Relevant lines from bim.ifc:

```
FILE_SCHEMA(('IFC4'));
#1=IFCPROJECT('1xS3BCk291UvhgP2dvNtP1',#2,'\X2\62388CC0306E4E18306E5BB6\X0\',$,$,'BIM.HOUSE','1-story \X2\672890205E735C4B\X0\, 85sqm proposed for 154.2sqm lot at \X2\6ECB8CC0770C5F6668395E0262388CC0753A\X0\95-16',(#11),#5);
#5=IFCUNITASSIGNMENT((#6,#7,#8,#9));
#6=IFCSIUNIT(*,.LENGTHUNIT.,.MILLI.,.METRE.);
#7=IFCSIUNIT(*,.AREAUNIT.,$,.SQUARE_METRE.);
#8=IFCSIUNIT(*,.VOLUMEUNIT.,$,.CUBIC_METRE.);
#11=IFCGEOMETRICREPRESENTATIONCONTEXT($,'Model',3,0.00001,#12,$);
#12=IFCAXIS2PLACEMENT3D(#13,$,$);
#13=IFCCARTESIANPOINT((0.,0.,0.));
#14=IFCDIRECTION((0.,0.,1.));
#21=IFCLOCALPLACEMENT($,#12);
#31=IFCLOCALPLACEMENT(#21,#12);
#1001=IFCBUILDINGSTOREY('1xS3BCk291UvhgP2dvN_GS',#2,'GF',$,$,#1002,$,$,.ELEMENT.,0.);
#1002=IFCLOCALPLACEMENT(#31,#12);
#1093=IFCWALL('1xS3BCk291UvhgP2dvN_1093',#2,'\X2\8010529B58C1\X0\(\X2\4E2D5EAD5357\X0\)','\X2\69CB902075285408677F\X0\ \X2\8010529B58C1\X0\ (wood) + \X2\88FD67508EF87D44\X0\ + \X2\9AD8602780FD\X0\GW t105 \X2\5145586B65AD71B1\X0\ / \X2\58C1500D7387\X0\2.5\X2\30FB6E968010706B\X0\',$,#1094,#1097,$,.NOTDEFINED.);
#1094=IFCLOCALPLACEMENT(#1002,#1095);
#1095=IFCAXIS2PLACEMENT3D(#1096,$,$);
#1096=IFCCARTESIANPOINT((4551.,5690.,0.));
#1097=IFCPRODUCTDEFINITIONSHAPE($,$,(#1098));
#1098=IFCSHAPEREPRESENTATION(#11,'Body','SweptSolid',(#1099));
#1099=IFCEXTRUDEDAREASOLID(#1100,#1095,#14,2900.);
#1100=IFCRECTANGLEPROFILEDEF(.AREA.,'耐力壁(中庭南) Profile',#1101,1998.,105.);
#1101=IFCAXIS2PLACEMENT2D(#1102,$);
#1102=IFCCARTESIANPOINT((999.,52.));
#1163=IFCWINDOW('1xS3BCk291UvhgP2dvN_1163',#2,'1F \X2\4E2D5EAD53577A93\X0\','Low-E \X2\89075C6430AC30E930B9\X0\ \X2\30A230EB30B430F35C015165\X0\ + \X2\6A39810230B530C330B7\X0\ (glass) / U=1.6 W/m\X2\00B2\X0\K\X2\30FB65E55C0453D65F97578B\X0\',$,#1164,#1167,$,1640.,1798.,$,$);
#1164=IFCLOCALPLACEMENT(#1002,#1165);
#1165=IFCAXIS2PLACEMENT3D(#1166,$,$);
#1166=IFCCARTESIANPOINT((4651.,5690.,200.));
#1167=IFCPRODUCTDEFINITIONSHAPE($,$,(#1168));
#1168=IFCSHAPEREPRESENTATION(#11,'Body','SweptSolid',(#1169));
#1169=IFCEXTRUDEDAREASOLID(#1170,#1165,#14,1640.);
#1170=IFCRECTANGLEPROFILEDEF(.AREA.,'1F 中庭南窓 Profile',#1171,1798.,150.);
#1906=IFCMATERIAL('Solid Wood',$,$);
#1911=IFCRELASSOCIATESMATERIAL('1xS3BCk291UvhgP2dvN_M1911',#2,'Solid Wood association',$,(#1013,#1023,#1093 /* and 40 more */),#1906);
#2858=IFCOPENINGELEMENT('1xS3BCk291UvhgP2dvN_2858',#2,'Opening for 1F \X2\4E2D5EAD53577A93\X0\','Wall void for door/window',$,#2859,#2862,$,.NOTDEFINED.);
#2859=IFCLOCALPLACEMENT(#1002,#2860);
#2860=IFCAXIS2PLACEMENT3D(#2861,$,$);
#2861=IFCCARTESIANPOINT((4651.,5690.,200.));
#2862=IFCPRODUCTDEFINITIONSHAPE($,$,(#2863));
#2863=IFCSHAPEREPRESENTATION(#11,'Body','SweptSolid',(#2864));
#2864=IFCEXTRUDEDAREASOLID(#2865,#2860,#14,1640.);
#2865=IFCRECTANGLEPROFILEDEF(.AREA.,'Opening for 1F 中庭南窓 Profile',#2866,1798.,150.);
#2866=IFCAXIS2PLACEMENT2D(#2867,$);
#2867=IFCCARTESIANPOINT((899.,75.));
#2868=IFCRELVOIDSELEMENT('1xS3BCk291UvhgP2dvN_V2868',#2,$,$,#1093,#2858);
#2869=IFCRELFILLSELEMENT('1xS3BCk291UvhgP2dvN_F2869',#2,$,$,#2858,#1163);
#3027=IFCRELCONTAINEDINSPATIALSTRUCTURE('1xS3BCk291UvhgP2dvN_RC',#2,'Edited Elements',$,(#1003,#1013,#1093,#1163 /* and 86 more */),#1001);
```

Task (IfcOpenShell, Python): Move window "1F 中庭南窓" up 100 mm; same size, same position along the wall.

```python
import numpy as np
import ifcopenshell
import ifcopenshell.api.geometry
import ifcopenshell.util.placement
import ifcopenshell.util.unit

model = ifcopenshell.open("bim.ifc")
unit_scale = ifcopenshell.util.unit.calculate_unit_scale(model)

window = model.by_guid("1xS3BCk291UvhgP2dvN_1163")
opening = window.FillsVoids[0].RelatingOpeningElement
dz = 100.0

shift = np.array([0.0, 0.0, dz])
# The window is not placed relative to its opening, so move both.
for product in (opening, window):
    matrix = ifcopenshell.util.placement.get_local_placement(product.ObjectPlacement)
    matrix[:3, 3] += shift
    ifcopenshell.api.geometry.edit_object_placement(model, product=product, matrix=matrix, is_si=False)

print(f"moved by {dz * unit_scale:+.3f} m")

model.write("bim_rev.ifc")
```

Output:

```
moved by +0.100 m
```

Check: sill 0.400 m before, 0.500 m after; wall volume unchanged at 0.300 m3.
